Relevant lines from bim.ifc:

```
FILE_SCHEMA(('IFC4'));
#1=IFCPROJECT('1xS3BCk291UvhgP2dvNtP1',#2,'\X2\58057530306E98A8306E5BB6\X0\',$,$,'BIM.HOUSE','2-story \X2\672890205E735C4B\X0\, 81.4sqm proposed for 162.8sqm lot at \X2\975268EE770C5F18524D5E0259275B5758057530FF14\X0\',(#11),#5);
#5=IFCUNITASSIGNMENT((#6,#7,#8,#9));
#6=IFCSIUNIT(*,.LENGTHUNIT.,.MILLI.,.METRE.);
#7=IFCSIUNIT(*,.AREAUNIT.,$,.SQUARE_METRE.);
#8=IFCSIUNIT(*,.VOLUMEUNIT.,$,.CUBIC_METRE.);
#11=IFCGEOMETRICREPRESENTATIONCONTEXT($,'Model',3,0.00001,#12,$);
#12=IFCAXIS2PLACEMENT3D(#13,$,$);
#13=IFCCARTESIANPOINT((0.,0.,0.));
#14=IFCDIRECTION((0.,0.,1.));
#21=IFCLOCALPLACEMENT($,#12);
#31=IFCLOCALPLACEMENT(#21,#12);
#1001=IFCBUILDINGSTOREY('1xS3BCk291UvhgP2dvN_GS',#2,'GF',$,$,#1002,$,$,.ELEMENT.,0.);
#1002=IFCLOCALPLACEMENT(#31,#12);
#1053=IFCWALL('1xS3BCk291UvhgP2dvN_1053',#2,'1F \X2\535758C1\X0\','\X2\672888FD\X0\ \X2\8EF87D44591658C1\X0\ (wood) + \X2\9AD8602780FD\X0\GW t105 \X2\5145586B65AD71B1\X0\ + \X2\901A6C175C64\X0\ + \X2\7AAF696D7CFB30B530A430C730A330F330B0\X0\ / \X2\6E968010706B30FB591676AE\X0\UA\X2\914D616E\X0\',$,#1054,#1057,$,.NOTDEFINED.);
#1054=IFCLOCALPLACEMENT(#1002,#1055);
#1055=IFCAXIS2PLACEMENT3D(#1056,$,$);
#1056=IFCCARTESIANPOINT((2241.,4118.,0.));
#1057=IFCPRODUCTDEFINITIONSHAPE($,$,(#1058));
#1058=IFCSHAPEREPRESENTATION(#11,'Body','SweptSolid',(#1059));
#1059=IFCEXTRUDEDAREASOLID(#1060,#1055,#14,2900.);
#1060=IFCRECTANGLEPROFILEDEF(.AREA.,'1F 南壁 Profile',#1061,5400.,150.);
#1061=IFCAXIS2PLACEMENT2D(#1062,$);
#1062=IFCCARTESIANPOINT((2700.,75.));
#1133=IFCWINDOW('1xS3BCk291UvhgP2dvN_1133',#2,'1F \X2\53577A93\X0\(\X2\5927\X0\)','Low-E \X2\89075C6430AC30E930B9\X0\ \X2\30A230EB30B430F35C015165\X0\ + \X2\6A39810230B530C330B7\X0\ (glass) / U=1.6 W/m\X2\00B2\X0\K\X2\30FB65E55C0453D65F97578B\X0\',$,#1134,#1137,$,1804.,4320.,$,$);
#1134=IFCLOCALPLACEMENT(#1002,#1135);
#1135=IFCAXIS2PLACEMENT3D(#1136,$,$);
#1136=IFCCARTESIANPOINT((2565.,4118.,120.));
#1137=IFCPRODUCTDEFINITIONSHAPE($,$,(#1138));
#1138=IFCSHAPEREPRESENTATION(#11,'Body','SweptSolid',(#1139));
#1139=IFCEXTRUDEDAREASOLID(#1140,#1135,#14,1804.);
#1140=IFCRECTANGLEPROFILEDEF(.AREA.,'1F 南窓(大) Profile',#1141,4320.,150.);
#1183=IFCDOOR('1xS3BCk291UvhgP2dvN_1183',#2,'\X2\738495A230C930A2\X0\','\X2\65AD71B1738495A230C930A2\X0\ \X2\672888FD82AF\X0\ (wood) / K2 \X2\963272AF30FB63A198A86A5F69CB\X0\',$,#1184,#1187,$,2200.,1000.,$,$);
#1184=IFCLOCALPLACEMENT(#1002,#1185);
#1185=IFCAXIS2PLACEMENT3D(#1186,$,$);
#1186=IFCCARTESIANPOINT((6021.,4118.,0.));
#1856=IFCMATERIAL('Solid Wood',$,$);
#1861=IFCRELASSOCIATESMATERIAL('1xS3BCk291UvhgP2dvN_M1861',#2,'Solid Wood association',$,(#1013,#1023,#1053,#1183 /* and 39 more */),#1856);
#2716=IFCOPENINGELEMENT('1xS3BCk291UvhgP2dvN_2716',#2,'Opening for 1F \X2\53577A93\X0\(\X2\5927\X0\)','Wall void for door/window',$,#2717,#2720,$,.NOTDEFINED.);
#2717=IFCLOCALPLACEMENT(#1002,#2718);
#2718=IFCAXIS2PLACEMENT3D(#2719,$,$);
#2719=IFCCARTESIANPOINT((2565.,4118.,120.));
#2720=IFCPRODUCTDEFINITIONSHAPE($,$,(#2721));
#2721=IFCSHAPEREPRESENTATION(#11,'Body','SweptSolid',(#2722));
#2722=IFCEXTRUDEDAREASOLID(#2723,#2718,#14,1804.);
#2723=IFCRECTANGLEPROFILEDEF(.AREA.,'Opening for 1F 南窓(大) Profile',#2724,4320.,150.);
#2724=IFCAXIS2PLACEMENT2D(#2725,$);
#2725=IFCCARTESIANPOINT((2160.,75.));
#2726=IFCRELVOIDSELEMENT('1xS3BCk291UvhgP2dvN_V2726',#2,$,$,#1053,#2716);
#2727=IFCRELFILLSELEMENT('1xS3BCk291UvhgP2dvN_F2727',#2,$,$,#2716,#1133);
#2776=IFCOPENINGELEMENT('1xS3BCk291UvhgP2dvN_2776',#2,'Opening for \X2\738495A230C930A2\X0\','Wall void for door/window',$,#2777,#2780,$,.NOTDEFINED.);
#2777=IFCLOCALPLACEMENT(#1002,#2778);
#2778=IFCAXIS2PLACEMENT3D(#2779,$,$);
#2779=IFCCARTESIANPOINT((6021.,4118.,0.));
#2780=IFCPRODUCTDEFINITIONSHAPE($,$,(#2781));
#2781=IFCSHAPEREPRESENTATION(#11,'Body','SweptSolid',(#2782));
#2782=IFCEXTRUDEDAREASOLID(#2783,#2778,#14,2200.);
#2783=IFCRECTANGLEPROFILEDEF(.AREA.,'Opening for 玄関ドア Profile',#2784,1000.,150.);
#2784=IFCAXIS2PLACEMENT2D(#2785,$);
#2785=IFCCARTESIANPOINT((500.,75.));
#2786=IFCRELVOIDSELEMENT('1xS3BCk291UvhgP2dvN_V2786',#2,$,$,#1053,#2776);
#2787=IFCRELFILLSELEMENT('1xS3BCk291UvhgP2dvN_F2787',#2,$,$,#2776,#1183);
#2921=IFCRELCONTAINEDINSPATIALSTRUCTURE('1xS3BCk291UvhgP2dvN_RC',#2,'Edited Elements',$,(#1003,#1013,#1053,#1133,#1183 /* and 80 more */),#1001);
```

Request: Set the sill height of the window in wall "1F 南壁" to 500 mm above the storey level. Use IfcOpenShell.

```python
import numpy as np
import ifcopenshell
import ifcopenshell.api.geometry
import ifcopenshell.geom
import ifcopenshell.util.element
import ifcopenshell.util.placement
import ifcopenshell.util.shape
import ifcopenshell.util.unit

model = ifcopenshell.open("bim.ifc")
unit_scale = ifcopenshell.util.unit.calculate_unit_scale(model)

window = model.by_guid("1xS3BCk291UvhgP2dvN_1133")
opening = window.FillsVoids[0].RelatingOpeningElement
storey = ifcopenshell.util.element.get_container(window, ifc_class="IfcBuildingStorey")
level = ifcopenshell.util.placement.get_local_placement(storey.ObjectPlacement)[2, 3]

# The opening's origin need not be at the sill, so measure its lowest point.
shape = ifcopenshell.geom.create_shape(ifcopenshell.geom.settings(), opening)
bottom = ifcopenshell.util.shape.get_shape_bottom_elevation(shape, shape.geometry) / unit_scale
dz = level + 500.0 - bottom

shift = np.array([0.0, 0.0, dz])
# The window is not placed relative to its opening, so move both.
for product in (opening, window):
    matrix = ifcopenshell.util.placement.get_local_placement(product.ObjectPlacement)
    matrix[:3, 3] += shift
    ifcopenshell.api.geometry.edit_object_placement(model, product=product, matrix=matrix, is_si=False)

print(f"moved by {dz * unit_scale:+.3f} m")

model.write("bim_updated.ifc")
```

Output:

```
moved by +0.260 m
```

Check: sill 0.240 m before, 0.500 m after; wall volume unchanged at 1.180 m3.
